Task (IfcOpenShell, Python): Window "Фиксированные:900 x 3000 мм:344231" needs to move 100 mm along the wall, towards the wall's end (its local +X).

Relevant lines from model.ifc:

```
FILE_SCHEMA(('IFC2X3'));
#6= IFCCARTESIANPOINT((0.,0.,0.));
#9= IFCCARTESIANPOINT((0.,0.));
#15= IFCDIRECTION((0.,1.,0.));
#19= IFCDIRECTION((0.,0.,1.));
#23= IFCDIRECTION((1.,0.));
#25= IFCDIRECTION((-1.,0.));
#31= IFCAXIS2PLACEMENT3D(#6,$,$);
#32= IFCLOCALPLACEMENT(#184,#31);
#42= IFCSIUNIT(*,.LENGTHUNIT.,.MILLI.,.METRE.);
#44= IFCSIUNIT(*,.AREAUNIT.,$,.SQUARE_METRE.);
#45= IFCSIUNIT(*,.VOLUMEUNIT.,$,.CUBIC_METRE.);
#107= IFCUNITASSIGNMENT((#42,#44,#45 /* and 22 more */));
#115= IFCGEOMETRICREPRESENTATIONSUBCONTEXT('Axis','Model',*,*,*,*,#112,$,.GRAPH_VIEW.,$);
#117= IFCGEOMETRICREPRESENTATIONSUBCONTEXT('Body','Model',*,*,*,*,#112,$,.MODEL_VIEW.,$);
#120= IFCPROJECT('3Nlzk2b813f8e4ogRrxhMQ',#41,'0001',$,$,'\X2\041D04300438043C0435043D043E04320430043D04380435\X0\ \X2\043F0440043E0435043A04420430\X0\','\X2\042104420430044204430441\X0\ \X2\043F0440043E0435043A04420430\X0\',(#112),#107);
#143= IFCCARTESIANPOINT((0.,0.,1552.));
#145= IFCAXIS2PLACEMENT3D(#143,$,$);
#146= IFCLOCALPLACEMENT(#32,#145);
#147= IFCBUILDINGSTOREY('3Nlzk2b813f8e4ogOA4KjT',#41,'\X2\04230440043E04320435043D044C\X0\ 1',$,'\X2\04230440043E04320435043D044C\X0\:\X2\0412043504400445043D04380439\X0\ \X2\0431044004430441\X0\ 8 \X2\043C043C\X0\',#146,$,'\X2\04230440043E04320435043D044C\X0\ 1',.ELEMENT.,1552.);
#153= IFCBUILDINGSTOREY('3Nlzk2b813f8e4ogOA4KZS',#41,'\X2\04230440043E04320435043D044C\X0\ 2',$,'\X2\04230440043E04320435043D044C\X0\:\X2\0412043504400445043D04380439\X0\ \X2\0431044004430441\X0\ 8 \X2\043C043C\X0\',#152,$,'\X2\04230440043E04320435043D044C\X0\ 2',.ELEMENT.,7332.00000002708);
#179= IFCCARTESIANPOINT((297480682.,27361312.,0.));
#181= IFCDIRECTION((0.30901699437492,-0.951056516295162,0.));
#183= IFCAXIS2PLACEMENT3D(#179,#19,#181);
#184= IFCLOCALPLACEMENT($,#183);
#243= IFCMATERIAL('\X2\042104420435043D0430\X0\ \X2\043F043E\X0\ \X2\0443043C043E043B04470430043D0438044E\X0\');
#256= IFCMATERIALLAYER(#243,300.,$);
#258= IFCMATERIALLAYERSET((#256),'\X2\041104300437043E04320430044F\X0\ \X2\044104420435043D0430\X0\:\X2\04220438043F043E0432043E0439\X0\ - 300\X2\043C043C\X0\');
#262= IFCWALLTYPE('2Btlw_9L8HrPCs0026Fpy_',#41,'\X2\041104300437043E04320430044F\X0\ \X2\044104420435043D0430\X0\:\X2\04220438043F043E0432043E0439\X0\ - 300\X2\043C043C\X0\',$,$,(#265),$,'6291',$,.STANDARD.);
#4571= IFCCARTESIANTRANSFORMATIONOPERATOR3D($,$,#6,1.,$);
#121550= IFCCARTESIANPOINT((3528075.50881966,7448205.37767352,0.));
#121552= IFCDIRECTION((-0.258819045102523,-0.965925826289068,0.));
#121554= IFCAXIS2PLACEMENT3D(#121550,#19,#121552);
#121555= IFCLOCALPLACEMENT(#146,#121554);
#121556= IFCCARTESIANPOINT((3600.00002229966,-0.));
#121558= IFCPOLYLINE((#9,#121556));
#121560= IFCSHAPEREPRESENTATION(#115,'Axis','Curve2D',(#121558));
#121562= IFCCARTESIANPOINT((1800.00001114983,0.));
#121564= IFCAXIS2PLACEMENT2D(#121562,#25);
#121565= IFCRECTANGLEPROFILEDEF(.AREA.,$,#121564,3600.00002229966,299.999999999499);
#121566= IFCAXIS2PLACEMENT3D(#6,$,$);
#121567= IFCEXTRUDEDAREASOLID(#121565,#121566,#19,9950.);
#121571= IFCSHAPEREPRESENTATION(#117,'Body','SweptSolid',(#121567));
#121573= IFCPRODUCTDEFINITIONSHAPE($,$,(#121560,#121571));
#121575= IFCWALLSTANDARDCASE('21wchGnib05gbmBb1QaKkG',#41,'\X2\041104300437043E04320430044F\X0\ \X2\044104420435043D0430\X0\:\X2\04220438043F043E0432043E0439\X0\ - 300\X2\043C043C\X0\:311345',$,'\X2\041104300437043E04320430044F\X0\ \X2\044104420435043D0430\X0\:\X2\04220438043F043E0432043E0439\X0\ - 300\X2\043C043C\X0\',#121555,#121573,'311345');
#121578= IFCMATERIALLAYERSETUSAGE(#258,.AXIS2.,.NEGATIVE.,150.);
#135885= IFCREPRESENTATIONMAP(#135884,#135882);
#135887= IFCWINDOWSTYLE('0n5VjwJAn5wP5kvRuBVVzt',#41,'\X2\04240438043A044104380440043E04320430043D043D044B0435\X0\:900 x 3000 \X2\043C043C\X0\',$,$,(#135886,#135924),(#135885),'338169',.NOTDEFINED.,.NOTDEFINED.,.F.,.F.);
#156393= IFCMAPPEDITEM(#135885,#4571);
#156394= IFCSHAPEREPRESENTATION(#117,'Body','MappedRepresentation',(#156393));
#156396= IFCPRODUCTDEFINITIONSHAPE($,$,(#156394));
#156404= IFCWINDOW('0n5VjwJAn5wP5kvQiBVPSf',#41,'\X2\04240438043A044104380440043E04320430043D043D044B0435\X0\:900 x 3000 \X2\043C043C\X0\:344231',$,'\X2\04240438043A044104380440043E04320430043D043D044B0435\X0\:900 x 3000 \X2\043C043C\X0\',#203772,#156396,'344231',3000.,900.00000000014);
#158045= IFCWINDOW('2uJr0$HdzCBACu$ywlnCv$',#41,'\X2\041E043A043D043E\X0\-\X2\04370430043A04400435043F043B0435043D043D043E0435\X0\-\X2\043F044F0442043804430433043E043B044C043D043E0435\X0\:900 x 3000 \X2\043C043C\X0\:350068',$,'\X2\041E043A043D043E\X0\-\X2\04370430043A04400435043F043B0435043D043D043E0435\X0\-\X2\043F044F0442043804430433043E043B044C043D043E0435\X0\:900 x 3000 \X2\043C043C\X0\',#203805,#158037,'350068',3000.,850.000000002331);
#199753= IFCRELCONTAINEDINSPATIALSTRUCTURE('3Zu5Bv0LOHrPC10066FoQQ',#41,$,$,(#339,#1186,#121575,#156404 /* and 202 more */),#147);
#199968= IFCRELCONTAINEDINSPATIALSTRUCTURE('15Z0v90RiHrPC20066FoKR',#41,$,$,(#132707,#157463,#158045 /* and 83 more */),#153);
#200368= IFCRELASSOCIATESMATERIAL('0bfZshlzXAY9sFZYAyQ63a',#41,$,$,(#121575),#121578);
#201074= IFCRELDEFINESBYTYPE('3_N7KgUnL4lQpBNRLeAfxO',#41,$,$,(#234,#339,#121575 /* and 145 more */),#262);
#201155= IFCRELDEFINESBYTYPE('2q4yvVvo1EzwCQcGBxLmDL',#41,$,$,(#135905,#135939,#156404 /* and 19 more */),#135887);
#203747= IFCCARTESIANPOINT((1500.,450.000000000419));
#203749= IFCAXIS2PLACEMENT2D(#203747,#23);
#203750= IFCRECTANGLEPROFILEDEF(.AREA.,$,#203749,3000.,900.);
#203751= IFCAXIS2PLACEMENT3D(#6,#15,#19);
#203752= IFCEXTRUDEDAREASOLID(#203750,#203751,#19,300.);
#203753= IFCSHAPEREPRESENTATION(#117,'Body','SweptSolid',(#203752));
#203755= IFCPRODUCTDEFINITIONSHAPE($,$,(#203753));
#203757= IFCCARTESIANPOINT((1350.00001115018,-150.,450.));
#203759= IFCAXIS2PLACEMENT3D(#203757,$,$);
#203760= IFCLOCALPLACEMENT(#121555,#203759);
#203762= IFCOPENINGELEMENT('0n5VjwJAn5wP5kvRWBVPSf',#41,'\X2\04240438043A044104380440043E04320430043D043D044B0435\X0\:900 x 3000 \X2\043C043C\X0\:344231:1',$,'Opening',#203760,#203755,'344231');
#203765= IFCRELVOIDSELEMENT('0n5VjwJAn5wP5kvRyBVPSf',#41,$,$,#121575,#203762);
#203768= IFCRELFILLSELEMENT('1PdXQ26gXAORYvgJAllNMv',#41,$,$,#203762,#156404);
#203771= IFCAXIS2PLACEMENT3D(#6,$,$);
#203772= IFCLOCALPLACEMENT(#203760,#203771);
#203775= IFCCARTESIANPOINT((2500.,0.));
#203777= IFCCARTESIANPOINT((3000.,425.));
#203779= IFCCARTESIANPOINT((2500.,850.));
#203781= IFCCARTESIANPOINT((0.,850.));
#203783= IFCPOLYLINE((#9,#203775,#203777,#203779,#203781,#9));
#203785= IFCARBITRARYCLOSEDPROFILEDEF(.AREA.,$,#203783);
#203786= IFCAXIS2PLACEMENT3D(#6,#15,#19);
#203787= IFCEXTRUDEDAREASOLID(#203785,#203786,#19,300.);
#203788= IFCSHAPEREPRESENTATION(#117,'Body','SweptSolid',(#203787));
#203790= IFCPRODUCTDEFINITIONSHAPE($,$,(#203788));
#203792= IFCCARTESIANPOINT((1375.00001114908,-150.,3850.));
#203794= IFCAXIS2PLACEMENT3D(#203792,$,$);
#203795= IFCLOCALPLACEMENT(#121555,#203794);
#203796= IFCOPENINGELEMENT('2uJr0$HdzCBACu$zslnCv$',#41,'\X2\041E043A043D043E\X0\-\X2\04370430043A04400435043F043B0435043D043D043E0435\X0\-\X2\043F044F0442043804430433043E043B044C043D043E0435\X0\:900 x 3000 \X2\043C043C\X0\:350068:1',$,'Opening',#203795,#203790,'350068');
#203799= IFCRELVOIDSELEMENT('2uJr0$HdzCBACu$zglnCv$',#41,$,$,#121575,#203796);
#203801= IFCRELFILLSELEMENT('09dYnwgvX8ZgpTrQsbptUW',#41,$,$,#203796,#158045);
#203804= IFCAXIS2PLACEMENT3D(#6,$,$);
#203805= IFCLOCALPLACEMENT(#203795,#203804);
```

```python
import ifcopenshell
import ifcopenshell.api.geometry
import ifcopenshell.util.placement

model = ifcopenshell.open("model.ifc")

window = model.by_id(156404)
opening = window.FillsVoids[0].RelatingOpeningElement
wall = opening.VoidsElements[0].RelatingBuildingElement

wall_matrix = ifcopenshell.util.placement.get_local_placement(wall.ObjectPlacement)
shift = wall_matrix[:3, 0] * 100.0
before = ifcopenshell.util.placement.get_local_placement(window.ObjectPlacement)[:3, 3].copy()

# The window is placed relative to its opening, so it follows when the opening moves.
matrix = ifcopenshell.util.placement.get_local_placement(opening.ObjectPlacement)
matrix[:3, 3] += shift
ifcopenshell.api.geometry.edit_object_placement(
    model, product=opening, matrix=matrix, is_si=False, should_transform_children=True
)

after = ifcopenshell.util.placement.get_local_placement(window.ObjectPlacement)[:3, 3]
print("window moved by", (after - before).round(3) + 0.0)

model.write("model_rev.ifc")
```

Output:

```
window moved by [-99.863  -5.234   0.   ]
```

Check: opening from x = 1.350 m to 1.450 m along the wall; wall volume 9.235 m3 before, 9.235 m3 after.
